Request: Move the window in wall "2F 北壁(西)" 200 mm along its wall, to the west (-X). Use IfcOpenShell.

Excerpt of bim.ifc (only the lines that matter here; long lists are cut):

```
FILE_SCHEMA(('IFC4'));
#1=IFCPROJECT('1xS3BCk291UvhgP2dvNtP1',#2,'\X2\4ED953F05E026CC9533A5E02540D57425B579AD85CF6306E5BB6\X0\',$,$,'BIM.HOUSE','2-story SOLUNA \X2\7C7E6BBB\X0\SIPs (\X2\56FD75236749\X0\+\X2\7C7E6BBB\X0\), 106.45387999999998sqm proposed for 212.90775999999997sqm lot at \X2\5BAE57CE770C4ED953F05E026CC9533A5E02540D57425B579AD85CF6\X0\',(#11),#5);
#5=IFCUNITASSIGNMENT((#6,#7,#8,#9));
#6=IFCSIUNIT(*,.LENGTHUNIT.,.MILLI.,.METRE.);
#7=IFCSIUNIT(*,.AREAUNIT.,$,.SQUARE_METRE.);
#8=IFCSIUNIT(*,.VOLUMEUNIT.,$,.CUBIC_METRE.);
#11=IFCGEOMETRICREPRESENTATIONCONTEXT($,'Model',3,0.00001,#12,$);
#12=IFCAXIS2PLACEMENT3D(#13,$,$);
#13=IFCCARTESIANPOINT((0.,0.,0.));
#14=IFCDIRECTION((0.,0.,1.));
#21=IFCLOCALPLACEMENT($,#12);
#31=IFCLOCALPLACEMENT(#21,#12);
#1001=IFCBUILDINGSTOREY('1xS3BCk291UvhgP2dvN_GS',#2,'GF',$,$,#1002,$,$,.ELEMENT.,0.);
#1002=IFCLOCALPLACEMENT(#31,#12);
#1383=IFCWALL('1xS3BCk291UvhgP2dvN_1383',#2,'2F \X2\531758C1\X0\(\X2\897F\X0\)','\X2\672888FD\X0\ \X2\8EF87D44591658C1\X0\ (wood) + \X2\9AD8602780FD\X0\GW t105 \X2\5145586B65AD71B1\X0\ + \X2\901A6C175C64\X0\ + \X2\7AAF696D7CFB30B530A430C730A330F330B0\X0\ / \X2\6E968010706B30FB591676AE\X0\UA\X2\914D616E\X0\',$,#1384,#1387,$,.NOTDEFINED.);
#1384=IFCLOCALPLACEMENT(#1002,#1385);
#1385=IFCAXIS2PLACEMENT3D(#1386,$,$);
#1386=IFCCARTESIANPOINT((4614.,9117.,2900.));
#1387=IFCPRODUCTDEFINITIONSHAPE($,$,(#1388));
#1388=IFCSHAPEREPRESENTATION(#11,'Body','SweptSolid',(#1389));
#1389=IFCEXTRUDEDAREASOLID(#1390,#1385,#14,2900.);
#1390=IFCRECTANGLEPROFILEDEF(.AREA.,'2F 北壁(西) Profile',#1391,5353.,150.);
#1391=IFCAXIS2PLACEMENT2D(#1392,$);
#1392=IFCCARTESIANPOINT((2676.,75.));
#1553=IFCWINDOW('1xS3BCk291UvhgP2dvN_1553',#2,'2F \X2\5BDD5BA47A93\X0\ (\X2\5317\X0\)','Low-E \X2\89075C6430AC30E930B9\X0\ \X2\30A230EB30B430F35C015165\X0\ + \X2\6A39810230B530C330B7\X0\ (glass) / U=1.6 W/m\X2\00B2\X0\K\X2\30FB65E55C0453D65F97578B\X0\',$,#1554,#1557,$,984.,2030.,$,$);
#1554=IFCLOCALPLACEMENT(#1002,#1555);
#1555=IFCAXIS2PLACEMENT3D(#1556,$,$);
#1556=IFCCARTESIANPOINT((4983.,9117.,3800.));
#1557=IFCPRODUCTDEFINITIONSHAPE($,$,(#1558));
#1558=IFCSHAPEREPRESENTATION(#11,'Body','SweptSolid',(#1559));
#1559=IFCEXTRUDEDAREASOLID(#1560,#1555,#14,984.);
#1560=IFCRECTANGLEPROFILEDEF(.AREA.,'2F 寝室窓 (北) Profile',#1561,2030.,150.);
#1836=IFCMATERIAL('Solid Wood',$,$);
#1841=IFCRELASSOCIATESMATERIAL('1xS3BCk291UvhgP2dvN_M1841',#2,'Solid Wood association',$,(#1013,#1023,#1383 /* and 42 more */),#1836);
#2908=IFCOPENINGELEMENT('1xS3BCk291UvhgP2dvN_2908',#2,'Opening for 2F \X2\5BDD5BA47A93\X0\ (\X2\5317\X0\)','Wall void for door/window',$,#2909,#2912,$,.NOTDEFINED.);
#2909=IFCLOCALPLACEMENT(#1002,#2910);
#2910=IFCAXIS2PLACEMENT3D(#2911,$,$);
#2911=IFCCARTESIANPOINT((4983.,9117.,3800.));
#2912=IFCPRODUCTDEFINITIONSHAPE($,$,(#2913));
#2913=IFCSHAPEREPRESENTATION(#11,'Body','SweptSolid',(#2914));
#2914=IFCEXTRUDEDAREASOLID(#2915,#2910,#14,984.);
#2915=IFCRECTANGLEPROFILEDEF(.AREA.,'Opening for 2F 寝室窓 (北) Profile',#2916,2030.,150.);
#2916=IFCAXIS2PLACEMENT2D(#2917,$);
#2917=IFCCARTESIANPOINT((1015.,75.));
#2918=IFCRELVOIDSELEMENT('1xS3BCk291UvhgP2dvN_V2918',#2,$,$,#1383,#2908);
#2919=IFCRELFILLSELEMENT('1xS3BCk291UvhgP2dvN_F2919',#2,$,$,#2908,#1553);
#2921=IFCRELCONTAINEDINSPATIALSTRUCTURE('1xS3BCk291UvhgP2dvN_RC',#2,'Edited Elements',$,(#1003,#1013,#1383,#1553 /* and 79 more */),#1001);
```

```python
import ifcopenshell
import ifcopenshell.api.geometry
import ifcopenshell.util.placement
import ifcopenshell.util.unit

model = ifcopenshell.open("bim.ifc")
unit_scale = ifcopenshell.util.unit.calculate_unit_scale(model)

window = model.by_guid("1xS3BCk291UvhgP2dvN_1553")
opening = window.FillsVoids[0].RelatingOpeningElement
wall = opening.VoidsElements[0].RelatingBuildingElement

wall_matrix = ifcopenshell.util.placement.get_local_placement(wall.ObjectPlacement)
shift = wall_matrix[:3, 0] * -0.2 / unit_scale
before = ifcopenshell.util.placement.get_local_placement(window.ObjectPlacement)[:3, 3].copy()

# The window is not placed relative to its opening, so move both.
for product in (opening, window):
    matrix = ifcopenshell.util.placement.get_local_placement(product.ObjectPlacement)
    matrix[:3, 3] += shift
    ifcopenshell.api.geometry.edit_object_placement(model, product=product, matrix=matrix, is_si=False)

after = ifcopenshell.util.placement.get_local_placement(window.ObjectPlacement)[:3, 3]
print("window moved by", (after - before).round(3) + 0.0)

model.write("bim_v2.ifc")
```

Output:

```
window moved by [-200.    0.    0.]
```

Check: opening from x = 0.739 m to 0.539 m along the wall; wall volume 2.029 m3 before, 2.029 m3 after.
